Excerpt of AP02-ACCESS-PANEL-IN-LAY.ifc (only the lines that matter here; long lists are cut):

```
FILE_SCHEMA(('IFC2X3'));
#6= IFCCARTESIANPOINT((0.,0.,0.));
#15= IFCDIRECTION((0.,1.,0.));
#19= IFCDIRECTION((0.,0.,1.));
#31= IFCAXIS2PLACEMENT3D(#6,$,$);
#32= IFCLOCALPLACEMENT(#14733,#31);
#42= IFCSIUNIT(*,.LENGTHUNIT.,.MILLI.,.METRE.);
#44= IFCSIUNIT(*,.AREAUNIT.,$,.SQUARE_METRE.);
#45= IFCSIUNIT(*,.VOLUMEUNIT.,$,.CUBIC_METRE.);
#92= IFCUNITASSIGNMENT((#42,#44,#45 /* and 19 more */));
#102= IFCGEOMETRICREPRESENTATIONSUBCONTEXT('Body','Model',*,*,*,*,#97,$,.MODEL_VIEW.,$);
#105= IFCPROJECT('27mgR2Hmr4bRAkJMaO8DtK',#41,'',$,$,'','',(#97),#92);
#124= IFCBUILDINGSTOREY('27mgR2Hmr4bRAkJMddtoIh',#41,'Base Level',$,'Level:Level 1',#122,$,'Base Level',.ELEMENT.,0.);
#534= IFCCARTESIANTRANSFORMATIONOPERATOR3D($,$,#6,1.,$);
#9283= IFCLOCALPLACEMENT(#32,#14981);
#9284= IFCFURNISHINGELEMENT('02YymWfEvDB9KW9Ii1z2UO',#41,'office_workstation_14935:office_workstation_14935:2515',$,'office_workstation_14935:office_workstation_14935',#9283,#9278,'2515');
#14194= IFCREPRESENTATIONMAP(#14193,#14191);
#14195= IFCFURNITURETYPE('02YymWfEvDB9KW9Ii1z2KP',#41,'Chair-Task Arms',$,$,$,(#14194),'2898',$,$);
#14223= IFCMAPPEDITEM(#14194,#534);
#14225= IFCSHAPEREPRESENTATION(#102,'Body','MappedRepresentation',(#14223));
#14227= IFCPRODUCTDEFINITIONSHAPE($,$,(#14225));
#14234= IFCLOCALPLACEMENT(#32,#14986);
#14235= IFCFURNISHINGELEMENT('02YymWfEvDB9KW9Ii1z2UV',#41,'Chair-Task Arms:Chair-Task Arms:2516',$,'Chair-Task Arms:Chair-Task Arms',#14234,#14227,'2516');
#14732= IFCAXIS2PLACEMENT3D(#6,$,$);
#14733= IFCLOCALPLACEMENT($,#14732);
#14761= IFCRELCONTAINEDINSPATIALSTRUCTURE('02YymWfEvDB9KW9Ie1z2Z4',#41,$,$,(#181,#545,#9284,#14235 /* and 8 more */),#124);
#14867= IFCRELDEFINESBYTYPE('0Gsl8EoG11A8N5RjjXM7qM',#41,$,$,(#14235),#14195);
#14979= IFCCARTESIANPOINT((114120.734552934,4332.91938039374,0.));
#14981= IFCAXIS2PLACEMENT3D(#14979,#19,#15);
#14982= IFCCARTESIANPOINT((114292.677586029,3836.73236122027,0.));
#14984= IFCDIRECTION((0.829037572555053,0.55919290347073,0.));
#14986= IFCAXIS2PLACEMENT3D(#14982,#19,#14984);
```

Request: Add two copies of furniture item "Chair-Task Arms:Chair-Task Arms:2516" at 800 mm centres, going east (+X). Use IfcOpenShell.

```python
import numpy as np
import ifcopenshell
import ifcopenshell.api.geometry
import ifcopenshell.api.root
import ifcopenshell.util.element
import ifcopenshell.util.placement
import ifcopenshell.util.unit

model = ifcopenshell.open("AP02-ACCESS-PANEL-IN-LAY.ifc")
unit_scale = ifcopenshell.util.unit.calculate_unit_scale(model)


def reuse_history(source, copy):
    """copy_class also copies each property set's owner history, people and application; keep the originals."""
    for rel in copy.IsDefinedBy:
        if rel.is_a("IfcRelDefinesByProperties") and (history := rel.RelatingPropertyDefinition.OwnerHistory):
            rel.RelatingPropertyDefinition.OwnerHistory = source.OwnerHistory
            ifcopenshell.util.element.remove_deep2(model, history)


source = model.by_guid("02YymWfEvDB9KW9Ii1z2UV")
base = ifcopenshell.util.placement.get_local_placement(source.ObjectPlacement)
step = np.array([1.0, 0.0, 0.0]) * 0.8 / unit_scale

for i in range(1, 3):
    copy = ifcopenshell.api.root.copy_class(model, product=source)
    copy.Representation = ifcopenshell.util.element.copy_deep(
        model, source.Representation, exclude=["IfcGeometricRepresentationContext", "IfcRepresentationMap"]
    )
    copy.Name = "Chair-Task Arms:Chair-Task Arms"
    copy.Tag = None
    reuse_history(source, copy)
    matrix = base.copy()
    matrix[:3, 3] += i * step
    print("added at", matrix[:3, 3].round(3) + 0.0)
    ifcopenshell.api.geometry.edit_object_placement(model, product=copy, matrix=matrix, is_si=False)

model.write("AP02-ACCESS-PANEL-IN-LAY_v2.ifc")
```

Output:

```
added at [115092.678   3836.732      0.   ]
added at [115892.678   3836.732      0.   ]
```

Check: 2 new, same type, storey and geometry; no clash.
